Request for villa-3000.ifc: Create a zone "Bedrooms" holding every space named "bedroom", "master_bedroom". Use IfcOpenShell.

First a look at what the model holds.

```python
import ifcopenshell

model = ifcopenshell.open("villa-3000.ifc")
print(model.schema)
seen = {}
for space in model.by_type("IfcSpace"):
    seen[space.LongName] = seen.get(space.LongName, 0) + 1
for name, count in sorted(seen.items(), key=str):
    print(count, "x", name)
print("zones:", [z.Name for z in model.by_type("IfcZone")][:20])
```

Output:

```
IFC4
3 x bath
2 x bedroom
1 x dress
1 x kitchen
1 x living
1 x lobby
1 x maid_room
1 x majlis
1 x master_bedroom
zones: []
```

```python
import ifcopenshell
import ifcopenshell.api.group
import ifcopenshell.api.root

model = ifcopenshell.open("villa-3000.ifc")

names = {"bedroom", "master_bedroom"}
spaces = [s for s in model.by_type("IfcSpace") if s.LongName in names]

zone = ifcopenshell.api.root.create_entity(model, ifc_class="IfcZone", name="Bedrooms")
ifcopenshell.api.group.assign_group(model, products=spaces, group=zone)
print(len(spaces), "spaces in", zone.Name)

model.write("villa-3000_rev.ifc")
```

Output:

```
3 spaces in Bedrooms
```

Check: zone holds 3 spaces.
